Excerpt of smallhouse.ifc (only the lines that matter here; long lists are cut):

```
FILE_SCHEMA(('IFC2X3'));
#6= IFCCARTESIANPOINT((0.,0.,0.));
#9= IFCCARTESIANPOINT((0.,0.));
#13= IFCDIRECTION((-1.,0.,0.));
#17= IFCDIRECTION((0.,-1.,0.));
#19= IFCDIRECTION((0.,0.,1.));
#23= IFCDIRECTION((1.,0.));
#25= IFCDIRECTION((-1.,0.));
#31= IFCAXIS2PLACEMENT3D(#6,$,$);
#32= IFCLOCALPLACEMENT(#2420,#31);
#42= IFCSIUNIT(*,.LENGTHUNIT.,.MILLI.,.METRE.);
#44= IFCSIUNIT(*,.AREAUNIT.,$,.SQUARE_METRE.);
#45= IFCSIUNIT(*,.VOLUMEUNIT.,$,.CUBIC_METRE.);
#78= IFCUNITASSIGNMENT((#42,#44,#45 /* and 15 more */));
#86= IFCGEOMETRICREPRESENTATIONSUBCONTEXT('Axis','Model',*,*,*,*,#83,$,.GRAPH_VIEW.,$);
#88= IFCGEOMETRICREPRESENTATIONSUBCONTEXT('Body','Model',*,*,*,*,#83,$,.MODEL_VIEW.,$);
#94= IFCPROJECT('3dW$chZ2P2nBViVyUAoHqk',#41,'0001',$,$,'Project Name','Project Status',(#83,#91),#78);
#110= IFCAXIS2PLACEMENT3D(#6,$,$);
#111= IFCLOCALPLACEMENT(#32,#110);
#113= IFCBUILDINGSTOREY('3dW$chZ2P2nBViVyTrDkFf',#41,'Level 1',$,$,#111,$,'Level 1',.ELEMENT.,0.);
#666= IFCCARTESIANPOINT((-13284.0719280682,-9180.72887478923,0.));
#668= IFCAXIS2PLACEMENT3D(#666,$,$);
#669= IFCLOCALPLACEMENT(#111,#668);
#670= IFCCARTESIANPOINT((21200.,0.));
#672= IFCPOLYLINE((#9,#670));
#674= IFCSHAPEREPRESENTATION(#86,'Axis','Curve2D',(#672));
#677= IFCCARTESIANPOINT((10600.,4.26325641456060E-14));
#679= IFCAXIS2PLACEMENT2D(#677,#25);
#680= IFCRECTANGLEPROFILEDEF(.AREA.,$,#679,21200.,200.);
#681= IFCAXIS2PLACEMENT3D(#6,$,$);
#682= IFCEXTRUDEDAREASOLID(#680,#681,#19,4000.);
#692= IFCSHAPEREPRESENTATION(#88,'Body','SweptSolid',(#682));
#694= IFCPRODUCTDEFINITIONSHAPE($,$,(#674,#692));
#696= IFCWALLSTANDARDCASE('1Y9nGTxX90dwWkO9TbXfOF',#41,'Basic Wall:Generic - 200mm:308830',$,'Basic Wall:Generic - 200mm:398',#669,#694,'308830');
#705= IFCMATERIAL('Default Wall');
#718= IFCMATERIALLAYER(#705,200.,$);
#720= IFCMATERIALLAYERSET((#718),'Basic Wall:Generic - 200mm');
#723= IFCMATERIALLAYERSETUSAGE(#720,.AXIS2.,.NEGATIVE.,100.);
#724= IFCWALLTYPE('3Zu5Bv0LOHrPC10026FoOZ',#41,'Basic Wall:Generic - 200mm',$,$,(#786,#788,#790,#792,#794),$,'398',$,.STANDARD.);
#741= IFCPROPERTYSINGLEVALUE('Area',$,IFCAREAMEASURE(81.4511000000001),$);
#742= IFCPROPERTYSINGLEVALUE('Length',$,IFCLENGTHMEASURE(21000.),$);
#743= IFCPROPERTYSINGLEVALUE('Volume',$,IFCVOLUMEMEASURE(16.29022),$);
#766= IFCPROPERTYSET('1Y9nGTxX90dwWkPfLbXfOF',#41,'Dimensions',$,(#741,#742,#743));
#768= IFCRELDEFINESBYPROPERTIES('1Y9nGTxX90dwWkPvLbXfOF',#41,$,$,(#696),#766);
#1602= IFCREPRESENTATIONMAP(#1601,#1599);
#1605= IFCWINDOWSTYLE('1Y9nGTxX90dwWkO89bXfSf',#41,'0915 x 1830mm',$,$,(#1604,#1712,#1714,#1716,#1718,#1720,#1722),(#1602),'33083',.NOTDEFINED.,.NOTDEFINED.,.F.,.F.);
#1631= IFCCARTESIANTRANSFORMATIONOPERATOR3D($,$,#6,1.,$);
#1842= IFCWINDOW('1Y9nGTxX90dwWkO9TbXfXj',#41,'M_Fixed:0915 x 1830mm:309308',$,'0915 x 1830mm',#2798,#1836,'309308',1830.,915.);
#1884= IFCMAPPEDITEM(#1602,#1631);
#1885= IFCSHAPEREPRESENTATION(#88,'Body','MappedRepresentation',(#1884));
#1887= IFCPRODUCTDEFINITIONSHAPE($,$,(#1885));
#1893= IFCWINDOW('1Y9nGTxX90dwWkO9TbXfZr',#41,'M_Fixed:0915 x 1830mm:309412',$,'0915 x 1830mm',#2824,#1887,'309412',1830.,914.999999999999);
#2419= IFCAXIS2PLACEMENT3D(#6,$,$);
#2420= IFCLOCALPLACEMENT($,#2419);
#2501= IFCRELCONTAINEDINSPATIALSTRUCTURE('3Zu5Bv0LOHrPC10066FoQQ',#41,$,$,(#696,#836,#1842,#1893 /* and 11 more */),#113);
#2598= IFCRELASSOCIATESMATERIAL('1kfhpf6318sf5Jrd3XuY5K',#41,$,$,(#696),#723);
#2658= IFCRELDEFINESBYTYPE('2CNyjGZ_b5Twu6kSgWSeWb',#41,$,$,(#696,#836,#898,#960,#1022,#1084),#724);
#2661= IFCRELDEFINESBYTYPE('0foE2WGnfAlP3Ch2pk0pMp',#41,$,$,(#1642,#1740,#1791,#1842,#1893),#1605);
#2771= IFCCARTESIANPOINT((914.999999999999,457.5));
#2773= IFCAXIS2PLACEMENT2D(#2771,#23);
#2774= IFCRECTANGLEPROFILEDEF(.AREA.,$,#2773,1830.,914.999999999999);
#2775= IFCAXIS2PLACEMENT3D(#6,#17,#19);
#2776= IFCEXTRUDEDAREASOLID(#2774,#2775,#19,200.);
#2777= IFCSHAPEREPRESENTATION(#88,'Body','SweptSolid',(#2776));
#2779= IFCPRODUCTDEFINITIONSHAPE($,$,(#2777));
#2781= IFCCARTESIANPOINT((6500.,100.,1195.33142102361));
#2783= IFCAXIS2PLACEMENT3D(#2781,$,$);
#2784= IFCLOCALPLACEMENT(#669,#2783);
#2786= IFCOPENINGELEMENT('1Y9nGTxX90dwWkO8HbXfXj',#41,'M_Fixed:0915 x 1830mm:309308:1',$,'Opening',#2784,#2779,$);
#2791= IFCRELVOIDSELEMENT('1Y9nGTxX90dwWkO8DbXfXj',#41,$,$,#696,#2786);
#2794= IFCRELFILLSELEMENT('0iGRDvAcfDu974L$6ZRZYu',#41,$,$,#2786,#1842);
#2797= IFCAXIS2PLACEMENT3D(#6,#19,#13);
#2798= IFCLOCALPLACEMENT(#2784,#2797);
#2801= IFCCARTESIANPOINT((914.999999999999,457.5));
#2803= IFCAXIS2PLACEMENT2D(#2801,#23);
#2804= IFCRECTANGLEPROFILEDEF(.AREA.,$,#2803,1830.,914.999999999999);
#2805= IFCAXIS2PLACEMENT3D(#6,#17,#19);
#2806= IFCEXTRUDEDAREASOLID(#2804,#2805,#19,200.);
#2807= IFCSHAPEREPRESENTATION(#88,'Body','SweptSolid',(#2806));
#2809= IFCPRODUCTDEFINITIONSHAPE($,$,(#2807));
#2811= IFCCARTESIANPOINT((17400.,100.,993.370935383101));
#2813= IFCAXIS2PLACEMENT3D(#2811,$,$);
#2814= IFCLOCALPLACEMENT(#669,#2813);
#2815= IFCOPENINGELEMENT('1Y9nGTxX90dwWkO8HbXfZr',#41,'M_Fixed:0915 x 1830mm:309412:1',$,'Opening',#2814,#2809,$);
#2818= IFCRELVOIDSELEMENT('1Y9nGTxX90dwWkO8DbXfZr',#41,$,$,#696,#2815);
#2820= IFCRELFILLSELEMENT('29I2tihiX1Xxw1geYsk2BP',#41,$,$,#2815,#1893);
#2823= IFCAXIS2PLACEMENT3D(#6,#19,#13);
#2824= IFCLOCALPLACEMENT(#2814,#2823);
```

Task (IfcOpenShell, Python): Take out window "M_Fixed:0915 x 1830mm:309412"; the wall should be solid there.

```python
import ifcopenshell
import ifcopenshell.api.feature
import ifcopenshell.api.pset
import ifcopenshell.api.root
import ifcopenshell.geom
import ifcopenshell.util.element
import ifcopenshell.util.shape
import ifcopenshell.util.unit

model = ifcopenshell.open("smallhouse.ifc")
area_scale = ifcopenshell.util.unit.calculate_unit_scale(model, "AREAUNIT")
volume_scale = ifcopenshell.util.unit.calculate_unit_scale(model, "VOLUMEUNIT")
settings = ifcopenshell.geom.settings()


def volume(element):
    """Net volume in cubic metres, openings subtracted."""
    shape = ifcopenshell.geom.create_shape(settings, element)
    return ifcopenshell.util.shape.get_volume(shape.geometry)


window = model.by_guid("1Y9nGTxX90dwWkO9TbXfZr")
opening = window.FillsVoids[0].RelatingOpeningElement
wall = opening.VoidsElements[0].RelatingBuildingElement
before = volume(wall)

ifcopenshell.api.root.remove_product(model, product=window)
ifcopenshell.api.feature.remove_feature(model, feature=opening)

after = volume(wall)
thickness = 0.2  # wall thickness in metres

# Update the wall's stored quantities.
pset = model.by_id(ifcopenshell.util.element.get_pset(wall, "Dimensions", should_inherit=False)["id"])
ifcopenshell.api.pset.edit_pset(model, pset=pset, properties={
    "Area": model.create_entity("IfcAreaMeasure", after / thickness / area_scale),
    "Volume": model.create_entity("IfcVolumeMeasure", after / volume_scale),
})

print(f"wall volume {before:.3f} -> {after:.3f} m3")

model.write("smallhouse_updated.ifc")
```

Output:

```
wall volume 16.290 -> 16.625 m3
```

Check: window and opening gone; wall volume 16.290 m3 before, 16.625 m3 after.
